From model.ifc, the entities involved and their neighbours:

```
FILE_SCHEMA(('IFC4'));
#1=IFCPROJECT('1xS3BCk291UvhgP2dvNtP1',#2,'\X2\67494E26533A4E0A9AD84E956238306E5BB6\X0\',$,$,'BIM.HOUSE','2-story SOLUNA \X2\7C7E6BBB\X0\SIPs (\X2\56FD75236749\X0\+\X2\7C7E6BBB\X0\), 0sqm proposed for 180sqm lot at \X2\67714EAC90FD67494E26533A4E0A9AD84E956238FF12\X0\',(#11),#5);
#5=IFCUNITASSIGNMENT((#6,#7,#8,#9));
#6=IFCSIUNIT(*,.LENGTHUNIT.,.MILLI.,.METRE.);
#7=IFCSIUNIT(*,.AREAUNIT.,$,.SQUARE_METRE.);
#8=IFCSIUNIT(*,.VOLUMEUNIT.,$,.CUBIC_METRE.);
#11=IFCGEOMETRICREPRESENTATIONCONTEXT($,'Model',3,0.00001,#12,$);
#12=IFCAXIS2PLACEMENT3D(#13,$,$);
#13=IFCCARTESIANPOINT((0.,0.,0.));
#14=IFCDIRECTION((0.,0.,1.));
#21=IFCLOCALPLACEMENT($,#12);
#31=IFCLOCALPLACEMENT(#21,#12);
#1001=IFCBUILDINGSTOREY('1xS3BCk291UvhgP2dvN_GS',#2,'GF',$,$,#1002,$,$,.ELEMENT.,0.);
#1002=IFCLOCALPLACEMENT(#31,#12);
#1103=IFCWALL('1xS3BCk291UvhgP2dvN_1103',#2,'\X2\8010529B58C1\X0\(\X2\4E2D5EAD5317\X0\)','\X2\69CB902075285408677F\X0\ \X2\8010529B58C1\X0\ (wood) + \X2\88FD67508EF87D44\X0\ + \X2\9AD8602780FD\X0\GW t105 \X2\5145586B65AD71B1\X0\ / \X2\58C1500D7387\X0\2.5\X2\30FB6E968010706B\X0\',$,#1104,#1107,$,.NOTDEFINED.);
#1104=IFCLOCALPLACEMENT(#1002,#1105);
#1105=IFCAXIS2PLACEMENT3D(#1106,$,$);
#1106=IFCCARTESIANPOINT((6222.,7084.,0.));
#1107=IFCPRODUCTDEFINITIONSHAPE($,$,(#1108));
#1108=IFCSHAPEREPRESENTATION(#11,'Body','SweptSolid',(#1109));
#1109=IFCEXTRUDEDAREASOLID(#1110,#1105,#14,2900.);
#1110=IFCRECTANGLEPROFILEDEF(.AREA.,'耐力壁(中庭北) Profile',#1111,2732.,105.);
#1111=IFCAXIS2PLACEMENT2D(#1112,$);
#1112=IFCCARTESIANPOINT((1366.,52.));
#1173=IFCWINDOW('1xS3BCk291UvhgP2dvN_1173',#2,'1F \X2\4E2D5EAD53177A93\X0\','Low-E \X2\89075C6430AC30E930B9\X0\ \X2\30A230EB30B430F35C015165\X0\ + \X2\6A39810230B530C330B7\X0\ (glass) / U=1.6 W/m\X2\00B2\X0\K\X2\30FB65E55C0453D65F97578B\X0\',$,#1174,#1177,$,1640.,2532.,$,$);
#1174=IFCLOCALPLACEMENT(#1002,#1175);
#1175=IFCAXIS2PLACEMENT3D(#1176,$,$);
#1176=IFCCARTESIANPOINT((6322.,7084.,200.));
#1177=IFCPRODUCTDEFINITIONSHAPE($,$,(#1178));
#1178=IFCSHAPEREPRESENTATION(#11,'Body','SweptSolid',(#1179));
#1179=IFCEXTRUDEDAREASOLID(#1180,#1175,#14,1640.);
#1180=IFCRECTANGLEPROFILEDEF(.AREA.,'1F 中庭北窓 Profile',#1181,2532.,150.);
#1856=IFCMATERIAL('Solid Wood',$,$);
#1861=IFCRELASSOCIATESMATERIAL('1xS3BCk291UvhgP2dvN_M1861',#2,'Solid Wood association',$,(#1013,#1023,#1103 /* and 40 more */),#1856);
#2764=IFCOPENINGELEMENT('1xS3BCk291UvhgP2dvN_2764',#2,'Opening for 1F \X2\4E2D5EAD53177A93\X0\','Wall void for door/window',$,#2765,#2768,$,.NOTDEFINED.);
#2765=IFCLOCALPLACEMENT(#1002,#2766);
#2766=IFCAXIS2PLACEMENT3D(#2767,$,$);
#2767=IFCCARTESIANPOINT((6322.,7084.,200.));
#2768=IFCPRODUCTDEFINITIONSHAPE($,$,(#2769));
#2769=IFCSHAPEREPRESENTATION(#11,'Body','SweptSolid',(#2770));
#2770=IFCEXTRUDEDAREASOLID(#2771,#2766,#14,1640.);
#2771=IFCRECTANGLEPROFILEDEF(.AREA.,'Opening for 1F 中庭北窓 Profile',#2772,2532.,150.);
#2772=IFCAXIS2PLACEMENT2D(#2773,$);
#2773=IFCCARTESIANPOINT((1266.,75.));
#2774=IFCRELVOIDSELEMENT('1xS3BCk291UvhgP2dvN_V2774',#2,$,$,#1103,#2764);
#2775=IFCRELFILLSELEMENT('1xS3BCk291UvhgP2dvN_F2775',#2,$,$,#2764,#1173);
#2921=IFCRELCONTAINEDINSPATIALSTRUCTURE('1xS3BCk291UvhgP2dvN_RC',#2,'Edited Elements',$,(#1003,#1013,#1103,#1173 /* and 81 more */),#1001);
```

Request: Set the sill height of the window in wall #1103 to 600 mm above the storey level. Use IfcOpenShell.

```python
import numpy as np
import ifcopenshell
import ifcopenshell.api.geometry
import ifcopenshell.geom
import ifcopenshell.util.element
import ifcopenshell.util.placement
import ifcopenshell.util.shape
import ifcopenshell.util.unit

model = ifcopenshell.open("model.ifc")
unit_scale = ifcopenshell.util.unit.calculate_unit_scale(model)

window = model.by_guid("1xS3BCk291UvhgP2dvN_1173")
opening = window.FillsVoids[0].RelatingOpeningElement
storey = ifcopenshell.util.element.get_container(window, ifc_class="IfcBuildingStorey")
level = ifcopenshell.util.placement.get_local_placement(storey.ObjectPlacement)[2, 3]

# The opening's origin need not be at the sill, so measure its lowest point.
shape = ifcopenshell.geom.create_shape(ifcopenshell.geom.settings(), opening)
bottom = ifcopenshell.util.shape.get_shape_bottom_elevation(shape, shape.geometry) / unit_scale
dz = level + 0.6 / unit_scale - bottom

shift = np.array([0.0, 0.0, dz])
# The window is not placed relative to its opening, so move both.
for product in (opening, window):
    matrix = ifcopenshell.util.placement.get_local_placement(product.ObjectPlacement)
    matrix[:3, 3] += shift
    ifcopenshell.api.geometry.edit_object_placement(model, product=product, matrix=matrix, is_si=False)

print(f"moved by {dz * unit_scale:+.3f} m")

model.write("model_rev.ifc")
```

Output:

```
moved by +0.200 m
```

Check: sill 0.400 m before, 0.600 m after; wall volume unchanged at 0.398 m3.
